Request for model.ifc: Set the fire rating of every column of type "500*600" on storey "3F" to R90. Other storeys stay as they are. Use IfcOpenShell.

First a look at what the model holds.

```python
import ifcopenshell
import ifcopenshell.util.element

model = ifcopenshell.open("model.ifc")
print(model.schema)
storey = next(s for s in model.by_type("IfcBuildingStorey") if s.Name == "3F")
columns = [e for e in ifcopenshell.util.element.get_decomposition(storey) if e.is_a("IfcColumn")]
seen = {}
for e in columns:
    element_type = ifcopenshell.util.element.get_type(e)
    key = (element_type.Name if element_type != e and element_type else None, ifcopenshell.util.element.get_pset(e, "Pset_ColumnCommon", "FireRating"))
    seen[key] = seen.get(key, 0) + 1
for (name, value), count in sorted(seen.items(), key=str):
    print(count, "x", name, "|", value)
```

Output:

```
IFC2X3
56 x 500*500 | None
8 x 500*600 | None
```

```python
import ifcopenshell
import ifcopenshell.api.pset
import ifcopenshell.util.element

model = ifcopenshell.open("model.ifc")

storey = next(s for s in model.by_type("IfcBuildingStorey") if s.Name == "3F")
columns = [e for e in ifcopenshell.util.element.get_decomposition(storey) if e.is_a("IfcColumn")]

count = 0
for e in columns:
    element_type = ifcopenshell.util.element.get_type(e)
    if element_type in (None, e) or element_type.Name != "500*600":
        continue
    # add_pset returns the element's existing set when there is one.
    pset = ifcopenshell.api.pset.add_pset(model, product=e, name="Pset_ColumnCommon")
    ifcopenshell.api.pset.edit_pset(model, pset=pset, properties={"FireRating": "R90"})
    count += 1

print(count, "columns updated")

model.write("model_updated.ifc")
```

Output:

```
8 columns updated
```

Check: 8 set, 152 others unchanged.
